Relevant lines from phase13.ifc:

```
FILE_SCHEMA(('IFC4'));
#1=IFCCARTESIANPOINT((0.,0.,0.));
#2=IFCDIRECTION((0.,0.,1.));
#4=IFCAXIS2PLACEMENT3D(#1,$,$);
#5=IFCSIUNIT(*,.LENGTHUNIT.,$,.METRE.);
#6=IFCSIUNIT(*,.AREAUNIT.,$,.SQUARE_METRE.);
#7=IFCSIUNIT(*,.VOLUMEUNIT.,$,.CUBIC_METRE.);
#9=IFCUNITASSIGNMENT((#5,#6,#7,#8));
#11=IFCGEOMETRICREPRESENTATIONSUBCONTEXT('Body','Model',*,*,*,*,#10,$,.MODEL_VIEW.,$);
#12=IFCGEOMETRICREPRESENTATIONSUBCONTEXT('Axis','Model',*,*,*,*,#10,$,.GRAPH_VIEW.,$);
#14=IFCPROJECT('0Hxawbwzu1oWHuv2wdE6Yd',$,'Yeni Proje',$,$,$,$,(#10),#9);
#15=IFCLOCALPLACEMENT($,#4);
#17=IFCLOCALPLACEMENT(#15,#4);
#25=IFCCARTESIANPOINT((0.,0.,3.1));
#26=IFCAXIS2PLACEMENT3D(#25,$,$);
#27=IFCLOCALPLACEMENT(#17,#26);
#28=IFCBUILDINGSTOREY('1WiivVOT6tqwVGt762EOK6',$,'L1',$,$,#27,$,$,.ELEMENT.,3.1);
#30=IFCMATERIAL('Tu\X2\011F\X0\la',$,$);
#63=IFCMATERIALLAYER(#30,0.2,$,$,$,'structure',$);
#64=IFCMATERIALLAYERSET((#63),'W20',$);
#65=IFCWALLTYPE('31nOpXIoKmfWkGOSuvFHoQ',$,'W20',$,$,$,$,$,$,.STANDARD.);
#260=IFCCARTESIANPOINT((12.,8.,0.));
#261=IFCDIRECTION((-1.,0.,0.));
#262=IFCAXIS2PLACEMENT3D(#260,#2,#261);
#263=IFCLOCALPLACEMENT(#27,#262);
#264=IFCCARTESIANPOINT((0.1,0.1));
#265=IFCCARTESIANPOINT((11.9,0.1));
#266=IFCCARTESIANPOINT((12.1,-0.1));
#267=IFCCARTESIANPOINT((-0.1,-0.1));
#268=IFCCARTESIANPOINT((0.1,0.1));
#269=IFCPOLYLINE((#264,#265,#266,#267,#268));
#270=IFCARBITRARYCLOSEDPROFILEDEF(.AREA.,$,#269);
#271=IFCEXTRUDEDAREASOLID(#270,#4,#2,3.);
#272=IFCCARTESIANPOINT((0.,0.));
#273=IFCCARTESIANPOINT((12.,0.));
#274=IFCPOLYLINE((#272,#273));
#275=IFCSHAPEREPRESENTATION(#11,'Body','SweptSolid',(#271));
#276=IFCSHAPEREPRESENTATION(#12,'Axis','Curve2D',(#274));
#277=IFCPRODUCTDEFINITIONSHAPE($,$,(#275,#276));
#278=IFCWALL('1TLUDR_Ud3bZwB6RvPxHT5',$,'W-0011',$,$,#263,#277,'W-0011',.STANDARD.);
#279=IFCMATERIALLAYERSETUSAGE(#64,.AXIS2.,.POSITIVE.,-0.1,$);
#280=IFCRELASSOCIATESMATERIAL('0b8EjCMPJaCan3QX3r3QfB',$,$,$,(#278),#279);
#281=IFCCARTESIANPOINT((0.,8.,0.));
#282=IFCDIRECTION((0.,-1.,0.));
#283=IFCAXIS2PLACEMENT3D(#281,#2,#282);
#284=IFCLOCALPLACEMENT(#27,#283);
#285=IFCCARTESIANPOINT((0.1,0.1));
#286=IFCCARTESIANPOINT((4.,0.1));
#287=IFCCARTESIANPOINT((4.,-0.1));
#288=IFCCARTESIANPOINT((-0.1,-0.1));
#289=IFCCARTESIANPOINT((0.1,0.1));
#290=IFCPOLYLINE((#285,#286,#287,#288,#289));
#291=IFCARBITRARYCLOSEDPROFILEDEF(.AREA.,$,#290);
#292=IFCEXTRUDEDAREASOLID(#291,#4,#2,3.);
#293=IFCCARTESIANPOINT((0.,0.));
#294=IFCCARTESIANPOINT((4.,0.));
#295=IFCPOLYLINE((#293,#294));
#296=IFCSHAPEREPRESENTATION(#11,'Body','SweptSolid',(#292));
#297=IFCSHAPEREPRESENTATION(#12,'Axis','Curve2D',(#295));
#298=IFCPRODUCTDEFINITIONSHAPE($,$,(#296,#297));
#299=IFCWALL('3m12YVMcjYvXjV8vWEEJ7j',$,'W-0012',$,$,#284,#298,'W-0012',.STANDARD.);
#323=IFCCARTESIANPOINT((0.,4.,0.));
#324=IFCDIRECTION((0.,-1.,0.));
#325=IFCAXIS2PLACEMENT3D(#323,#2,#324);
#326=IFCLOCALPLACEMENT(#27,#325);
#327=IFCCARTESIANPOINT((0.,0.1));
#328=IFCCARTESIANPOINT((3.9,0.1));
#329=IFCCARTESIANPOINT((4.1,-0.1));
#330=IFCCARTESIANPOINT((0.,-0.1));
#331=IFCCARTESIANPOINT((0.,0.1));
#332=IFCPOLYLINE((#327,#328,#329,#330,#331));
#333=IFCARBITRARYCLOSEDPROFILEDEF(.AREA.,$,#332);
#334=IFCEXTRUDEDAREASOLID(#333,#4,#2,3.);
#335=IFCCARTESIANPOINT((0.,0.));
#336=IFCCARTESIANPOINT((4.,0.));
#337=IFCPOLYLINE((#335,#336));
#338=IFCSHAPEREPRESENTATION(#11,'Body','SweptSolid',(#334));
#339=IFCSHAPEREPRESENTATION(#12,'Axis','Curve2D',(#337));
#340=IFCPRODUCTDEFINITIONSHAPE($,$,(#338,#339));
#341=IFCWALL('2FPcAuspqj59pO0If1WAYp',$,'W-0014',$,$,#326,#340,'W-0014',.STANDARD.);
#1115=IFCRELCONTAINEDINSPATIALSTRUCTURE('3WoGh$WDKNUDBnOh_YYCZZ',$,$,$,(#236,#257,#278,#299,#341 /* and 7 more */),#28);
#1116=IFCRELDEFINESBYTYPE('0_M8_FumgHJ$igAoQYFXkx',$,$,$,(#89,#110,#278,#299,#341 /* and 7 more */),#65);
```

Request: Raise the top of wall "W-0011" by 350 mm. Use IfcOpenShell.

```python
import ifcopenshell
import ifcopenshell.geom
import ifcopenshell.util.representation
import ifcopenshell.util.shape
import ifcopenshell.util.unit

model = ifcopenshell.open("phase13.ifc")
unit_scale = ifcopenshell.util.unit.calculate_unit_scale(model)
settings = ifcopenshell.geom.settings()


def volume(element):
    """Net volume in cubic metres, openings subtracted."""
    shape = ifcopenshell.geom.create_shape(settings, element)
    return ifcopenshell.util.shape.get_volume(shape.geometry)


wall = model.by_id(278)
before = volume(wall)

body = ifcopenshell.util.representation.get_representation(wall, "Model", "Body")
solid = body.Items[0]
old_height = solid.Depth
solid.Depth += 0.35 / unit_scale
after = volume(wall)

print(f"height {old_height:g} -> {solid.Depth:g}, volume {before:.3f} -> {after:.3f} m3")

model.write("phase13-out.ifc")
```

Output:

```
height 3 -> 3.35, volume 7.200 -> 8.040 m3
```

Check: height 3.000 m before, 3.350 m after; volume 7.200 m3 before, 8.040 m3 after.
